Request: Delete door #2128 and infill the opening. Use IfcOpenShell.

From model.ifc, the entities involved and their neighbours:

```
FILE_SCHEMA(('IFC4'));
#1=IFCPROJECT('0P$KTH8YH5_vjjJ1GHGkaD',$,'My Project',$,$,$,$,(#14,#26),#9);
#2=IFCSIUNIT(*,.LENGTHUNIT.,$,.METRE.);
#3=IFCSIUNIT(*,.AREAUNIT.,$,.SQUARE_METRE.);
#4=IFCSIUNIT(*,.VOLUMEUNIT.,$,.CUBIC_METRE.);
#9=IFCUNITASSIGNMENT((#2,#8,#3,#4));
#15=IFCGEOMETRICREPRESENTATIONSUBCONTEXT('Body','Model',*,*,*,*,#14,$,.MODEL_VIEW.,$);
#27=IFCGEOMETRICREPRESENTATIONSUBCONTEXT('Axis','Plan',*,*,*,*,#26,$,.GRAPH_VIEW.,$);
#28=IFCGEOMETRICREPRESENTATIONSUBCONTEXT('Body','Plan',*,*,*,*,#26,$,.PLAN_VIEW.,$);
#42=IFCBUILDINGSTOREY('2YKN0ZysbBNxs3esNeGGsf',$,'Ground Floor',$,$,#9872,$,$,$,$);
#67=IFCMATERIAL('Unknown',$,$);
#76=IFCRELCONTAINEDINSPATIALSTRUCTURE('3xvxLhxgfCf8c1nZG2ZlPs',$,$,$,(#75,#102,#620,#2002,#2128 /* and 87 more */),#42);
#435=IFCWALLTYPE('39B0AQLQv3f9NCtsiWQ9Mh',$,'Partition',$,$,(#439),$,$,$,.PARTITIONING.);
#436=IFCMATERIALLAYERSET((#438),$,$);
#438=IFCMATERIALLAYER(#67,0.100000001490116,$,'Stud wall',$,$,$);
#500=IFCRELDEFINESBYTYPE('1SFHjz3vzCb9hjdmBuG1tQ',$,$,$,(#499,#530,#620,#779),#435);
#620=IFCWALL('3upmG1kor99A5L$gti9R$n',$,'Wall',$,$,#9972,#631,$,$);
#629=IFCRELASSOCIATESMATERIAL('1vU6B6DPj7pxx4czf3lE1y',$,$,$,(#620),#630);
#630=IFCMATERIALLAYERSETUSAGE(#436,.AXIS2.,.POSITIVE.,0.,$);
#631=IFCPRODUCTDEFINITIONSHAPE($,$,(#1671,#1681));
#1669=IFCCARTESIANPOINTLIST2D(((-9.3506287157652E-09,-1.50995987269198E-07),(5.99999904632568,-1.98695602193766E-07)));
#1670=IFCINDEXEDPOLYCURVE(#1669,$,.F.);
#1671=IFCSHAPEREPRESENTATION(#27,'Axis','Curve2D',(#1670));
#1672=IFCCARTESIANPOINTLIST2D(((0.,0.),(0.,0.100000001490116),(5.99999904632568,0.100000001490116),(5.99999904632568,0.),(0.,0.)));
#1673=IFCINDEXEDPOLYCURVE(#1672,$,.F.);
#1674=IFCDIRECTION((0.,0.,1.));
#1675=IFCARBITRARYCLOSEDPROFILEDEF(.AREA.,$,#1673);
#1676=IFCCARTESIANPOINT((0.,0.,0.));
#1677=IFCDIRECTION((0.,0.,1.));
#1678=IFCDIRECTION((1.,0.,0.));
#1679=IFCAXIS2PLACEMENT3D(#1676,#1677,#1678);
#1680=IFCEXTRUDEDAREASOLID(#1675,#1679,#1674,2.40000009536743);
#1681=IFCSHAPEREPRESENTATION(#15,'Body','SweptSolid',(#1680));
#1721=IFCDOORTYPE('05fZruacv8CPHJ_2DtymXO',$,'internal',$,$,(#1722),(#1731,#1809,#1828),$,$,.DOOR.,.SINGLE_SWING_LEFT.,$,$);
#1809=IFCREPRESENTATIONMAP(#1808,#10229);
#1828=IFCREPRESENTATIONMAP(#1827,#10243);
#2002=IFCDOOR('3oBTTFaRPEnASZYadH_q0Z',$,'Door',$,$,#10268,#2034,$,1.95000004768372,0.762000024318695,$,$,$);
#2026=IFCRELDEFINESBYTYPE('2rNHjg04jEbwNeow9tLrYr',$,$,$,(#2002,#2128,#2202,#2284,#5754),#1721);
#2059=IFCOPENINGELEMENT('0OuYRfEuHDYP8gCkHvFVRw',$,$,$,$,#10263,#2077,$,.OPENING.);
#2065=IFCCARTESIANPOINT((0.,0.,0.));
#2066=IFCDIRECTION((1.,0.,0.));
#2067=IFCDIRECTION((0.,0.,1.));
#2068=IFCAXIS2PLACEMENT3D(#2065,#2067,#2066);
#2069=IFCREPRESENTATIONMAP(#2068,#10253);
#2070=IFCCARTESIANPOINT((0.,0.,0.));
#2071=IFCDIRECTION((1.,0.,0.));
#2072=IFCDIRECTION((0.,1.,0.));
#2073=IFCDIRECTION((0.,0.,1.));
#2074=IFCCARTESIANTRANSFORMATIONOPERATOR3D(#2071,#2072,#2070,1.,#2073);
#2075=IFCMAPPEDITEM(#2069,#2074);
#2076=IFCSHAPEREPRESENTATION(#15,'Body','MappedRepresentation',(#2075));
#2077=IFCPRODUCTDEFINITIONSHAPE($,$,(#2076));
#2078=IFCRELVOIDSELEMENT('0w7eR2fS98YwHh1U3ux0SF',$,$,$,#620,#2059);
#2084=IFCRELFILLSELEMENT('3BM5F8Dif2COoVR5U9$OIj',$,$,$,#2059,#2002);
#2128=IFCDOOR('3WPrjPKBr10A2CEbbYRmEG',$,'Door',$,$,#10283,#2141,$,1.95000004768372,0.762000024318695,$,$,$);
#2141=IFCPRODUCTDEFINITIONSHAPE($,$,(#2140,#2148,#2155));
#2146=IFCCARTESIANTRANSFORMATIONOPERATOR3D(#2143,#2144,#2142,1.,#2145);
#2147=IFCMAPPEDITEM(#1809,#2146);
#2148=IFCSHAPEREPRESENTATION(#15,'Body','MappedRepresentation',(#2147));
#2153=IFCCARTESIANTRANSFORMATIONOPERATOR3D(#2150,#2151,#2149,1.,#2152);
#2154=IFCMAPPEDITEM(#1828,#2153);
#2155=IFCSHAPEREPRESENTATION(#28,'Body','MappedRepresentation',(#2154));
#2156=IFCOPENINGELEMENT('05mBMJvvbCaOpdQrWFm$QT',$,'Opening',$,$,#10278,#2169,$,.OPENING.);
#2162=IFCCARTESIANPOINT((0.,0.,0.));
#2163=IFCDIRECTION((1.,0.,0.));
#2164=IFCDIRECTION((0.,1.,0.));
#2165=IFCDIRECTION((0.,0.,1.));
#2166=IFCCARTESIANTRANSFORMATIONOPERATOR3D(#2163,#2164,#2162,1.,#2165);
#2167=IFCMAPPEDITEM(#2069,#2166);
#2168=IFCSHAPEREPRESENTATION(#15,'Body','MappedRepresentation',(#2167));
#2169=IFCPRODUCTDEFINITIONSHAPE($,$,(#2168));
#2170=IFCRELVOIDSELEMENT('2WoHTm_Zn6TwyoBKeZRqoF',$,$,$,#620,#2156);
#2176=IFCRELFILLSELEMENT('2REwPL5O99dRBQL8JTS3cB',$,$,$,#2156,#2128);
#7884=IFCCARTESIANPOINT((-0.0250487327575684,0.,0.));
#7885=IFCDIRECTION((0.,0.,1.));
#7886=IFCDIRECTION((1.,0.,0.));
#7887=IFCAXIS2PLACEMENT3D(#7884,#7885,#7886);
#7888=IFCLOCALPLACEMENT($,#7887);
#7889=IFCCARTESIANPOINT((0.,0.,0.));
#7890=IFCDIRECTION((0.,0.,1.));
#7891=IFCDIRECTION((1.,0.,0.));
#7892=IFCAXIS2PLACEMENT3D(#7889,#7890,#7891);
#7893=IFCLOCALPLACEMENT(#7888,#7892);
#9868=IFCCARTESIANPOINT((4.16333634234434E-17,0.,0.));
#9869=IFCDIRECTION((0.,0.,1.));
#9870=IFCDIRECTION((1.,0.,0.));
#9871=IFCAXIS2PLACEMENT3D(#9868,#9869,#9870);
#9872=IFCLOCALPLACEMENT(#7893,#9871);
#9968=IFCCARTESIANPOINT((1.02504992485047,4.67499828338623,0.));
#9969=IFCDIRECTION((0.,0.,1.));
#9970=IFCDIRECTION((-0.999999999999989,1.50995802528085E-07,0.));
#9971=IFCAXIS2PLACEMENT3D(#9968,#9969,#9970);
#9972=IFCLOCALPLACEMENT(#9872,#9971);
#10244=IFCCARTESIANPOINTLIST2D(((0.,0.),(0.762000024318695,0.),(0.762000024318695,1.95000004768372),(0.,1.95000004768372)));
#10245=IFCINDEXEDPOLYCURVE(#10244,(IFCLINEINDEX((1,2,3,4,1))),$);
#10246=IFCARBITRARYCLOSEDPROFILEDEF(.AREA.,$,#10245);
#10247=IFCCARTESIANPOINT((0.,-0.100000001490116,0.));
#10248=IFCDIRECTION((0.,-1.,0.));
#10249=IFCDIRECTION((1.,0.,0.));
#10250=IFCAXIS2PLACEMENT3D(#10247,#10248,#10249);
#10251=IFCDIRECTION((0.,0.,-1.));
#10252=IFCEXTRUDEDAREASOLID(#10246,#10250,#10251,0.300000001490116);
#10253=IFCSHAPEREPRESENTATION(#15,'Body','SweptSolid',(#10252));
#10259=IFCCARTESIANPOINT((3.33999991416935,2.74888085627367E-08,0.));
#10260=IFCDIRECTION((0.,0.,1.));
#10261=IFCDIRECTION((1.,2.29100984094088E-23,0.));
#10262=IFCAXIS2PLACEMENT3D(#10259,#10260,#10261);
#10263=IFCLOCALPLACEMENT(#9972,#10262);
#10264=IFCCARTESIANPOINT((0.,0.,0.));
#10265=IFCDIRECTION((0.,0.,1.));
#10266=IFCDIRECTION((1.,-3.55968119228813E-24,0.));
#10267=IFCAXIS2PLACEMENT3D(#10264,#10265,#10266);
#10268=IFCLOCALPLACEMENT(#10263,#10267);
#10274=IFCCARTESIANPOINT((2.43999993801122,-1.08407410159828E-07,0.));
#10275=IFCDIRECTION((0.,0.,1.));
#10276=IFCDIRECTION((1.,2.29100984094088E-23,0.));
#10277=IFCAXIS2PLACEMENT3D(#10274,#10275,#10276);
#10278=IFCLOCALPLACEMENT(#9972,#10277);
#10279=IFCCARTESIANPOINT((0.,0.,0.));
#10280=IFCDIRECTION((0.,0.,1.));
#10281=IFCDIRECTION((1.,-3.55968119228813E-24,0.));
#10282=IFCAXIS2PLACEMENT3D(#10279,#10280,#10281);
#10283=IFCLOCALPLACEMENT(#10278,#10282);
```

```python
import ifcopenshell
import ifcopenshell.api.feature
import ifcopenshell.api.root
import ifcopenshell.geom
import ifcopenshell.util.shape

model = ifcopenshell.open("model.ifc")
settings = ifcopenshell.geom.settings()


def volume(element):
    """Net volume in cubic metres, openings subtracted."""
    shape = ifcopenshell.geom.create_shape(settings, element)
    return ifcopenshell.util.shape.get_volume(shape.geometry)


door = model.by_id(2128)
opening = door.FillsVoids[0].RelatingOpeningElement
wall = opening.VoidsElements[0].RelatingBuildingElement
before = volume(wall)

ifcopenshell.api.root.remove_product(model, product=door)
ifcopenshell.api.feature.remove_feature(model, feature=opening)

after = volume(wall)

print(f"wall volume {before:.3f} -> {after:.3f} m3")

model.write("model_updated.ifc")
```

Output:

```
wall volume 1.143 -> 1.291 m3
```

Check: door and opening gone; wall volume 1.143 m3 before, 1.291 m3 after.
